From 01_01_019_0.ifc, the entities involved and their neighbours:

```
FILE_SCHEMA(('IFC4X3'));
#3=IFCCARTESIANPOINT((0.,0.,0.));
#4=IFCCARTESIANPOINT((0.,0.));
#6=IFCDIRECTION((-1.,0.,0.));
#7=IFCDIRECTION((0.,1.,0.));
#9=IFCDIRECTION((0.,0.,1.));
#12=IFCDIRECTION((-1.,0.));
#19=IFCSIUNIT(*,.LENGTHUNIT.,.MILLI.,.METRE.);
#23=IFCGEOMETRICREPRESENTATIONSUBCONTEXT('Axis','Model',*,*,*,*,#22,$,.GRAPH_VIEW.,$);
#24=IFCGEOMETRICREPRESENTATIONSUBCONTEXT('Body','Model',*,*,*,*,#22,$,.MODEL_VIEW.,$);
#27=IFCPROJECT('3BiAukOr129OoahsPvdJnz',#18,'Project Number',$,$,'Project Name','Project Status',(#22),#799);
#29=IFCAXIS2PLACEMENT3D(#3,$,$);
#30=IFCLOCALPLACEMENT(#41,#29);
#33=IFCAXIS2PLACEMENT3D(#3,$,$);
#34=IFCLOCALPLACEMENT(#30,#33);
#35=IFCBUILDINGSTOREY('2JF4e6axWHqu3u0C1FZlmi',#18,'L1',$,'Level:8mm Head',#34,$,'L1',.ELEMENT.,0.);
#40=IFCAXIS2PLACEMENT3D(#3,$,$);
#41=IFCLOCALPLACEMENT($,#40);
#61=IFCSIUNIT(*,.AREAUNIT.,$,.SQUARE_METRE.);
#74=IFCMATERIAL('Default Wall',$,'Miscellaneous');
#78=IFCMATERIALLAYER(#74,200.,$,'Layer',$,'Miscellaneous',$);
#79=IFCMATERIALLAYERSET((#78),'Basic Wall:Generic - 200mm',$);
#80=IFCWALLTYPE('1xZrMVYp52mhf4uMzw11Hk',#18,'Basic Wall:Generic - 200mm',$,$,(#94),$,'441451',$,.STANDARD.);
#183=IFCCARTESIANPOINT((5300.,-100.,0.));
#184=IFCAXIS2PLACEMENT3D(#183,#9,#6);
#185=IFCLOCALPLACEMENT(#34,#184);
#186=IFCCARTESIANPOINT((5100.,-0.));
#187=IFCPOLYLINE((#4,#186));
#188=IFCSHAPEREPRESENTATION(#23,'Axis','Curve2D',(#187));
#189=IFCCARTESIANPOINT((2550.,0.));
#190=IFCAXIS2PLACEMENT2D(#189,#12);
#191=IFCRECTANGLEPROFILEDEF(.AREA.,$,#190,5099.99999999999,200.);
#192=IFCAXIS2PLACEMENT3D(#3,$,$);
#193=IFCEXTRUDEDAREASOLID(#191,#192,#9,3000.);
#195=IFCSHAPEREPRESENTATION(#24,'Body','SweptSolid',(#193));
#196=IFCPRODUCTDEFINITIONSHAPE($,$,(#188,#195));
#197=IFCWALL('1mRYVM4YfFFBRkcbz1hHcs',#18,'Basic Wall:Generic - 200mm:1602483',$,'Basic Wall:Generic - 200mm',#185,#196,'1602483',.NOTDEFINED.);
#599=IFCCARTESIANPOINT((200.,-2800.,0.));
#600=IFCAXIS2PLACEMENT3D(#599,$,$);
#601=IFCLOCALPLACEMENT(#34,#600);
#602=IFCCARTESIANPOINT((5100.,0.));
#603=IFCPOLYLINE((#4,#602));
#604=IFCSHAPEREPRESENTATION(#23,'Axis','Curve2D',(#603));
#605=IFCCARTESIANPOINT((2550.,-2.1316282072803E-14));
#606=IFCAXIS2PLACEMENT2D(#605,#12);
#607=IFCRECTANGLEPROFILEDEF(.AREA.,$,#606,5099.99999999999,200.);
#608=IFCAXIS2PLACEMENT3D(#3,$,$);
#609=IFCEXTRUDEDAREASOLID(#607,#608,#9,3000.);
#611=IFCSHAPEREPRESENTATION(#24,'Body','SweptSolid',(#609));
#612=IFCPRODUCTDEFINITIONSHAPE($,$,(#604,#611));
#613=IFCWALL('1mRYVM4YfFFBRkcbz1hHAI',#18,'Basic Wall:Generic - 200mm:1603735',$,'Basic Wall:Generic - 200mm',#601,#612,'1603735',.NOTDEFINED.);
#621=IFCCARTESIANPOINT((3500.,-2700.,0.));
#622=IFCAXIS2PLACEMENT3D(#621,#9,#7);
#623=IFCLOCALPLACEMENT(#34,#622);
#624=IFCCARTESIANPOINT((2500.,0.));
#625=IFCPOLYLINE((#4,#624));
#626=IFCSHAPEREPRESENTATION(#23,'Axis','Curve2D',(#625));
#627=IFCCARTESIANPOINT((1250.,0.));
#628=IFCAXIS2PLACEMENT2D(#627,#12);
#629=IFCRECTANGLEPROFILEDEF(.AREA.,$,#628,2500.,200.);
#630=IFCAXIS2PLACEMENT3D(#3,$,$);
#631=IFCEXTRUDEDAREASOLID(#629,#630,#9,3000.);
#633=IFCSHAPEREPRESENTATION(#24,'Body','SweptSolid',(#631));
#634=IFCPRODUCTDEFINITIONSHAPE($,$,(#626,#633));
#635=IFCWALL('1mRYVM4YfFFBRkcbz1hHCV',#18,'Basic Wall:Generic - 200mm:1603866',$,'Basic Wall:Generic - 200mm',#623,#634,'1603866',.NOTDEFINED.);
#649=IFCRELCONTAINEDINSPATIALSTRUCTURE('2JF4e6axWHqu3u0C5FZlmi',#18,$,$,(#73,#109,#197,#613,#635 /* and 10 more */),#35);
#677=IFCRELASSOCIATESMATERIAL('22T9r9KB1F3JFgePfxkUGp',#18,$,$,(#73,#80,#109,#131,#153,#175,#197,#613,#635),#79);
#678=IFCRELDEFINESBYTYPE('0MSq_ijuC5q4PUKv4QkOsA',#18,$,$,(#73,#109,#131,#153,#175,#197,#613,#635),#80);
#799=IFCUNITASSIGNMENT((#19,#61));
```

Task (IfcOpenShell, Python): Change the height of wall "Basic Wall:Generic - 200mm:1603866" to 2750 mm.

```python
import ifcopenshell
import ifcopenshell.geom
import ifcopenshell.util.representation
import ifcopenshell.util.shape

model = ifcopenshell.open("01_01_019_0.ifc")
settings = ifcopenshell.geom.settings()


def volume(element):
    """Net volume in cubic metres, openings subtracted."""
    shape = ifcopenshell.geom.create_shape(settings, element)
    return ifcopenshell.util.shape.get_volume(shape.geometry)


wall = model.by_guid("1mRYVM4YfFFBRkcbz1hHCV")
before = volume(wall)

body = ifcopenshell.util.representation.get_representation(wall, "Model", "Body")
solid = body.Items[0]
old_height = solid.Depth
solid.Depth = 2750.0
after = volume(wall)

print(f"height {old_height:g} -> {solid.Depth:g}, volume {before:.3f} -> {after:.3f} m3")

model.write("01_01_019_0_v2.ifc")
```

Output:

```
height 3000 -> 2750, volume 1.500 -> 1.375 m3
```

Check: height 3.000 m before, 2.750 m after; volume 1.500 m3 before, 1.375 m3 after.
